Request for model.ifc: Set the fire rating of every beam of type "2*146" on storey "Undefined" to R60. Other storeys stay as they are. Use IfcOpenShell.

First a look at what the model holds.

```python
import ifcopenshell
import ifcopenshell.util.element

model = ifcopenshell.open("model.ifc")
print(model.schema)
storey = next(s for s in model.by_type("IfcBuildingStorey") if s.Name == "Undefined")
beams = [e for e in ifcopenshell.util.element.get_decomposition(storey) if e.is_a("IfcBeam")]
seen = {}
for e in beams:
    element_type = ifcopenshell.util.element.get_type(e)
    key = (element_type.Name if element_type != e and element_type else None, ifcopenshell.util.element.get_pset(e, "Pset_BeamCommon", "FireRating"))
    seen[key] = seen.get(key, 0) + 1
for (name, value), count in sorted(seen.items(), key=str):
    print(count, "x", name, "|", value)
```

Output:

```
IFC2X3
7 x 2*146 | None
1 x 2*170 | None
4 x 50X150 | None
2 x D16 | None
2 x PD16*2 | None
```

```python
import ifcopenshell
import ifcopenshell.api.pset
import ifcopenshell.util.element

model = ifcopenshell.open("model.ifc")

storey = next(s for s in model.by_type("IfcBuildingStorey") if s.Name == "Undefined")
beams = [e for e in ifcopenshell.util.element.get_decomposition(storey) if e.is_a("IfcBeam")]

count = 0
for e in beams:
    element_type = ifcopenshell.util.element.get_type(e)
    if element_type in (None, e) or element_type.Name != "2*146":
        continue
    # add_pset returns the element's existing set when there is one.
    pset = ifcopenshell.api.pset.add_pset(model, product=e, name="Pset_BeamCommon")
    ifcopenshell.api.pset.edit_pset(model, pset=pset, properties={"FireRating": "R60"})
    count += 1

print(count, "beams updated")

model.write("model_updated.ifc")
```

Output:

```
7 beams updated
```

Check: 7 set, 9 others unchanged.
